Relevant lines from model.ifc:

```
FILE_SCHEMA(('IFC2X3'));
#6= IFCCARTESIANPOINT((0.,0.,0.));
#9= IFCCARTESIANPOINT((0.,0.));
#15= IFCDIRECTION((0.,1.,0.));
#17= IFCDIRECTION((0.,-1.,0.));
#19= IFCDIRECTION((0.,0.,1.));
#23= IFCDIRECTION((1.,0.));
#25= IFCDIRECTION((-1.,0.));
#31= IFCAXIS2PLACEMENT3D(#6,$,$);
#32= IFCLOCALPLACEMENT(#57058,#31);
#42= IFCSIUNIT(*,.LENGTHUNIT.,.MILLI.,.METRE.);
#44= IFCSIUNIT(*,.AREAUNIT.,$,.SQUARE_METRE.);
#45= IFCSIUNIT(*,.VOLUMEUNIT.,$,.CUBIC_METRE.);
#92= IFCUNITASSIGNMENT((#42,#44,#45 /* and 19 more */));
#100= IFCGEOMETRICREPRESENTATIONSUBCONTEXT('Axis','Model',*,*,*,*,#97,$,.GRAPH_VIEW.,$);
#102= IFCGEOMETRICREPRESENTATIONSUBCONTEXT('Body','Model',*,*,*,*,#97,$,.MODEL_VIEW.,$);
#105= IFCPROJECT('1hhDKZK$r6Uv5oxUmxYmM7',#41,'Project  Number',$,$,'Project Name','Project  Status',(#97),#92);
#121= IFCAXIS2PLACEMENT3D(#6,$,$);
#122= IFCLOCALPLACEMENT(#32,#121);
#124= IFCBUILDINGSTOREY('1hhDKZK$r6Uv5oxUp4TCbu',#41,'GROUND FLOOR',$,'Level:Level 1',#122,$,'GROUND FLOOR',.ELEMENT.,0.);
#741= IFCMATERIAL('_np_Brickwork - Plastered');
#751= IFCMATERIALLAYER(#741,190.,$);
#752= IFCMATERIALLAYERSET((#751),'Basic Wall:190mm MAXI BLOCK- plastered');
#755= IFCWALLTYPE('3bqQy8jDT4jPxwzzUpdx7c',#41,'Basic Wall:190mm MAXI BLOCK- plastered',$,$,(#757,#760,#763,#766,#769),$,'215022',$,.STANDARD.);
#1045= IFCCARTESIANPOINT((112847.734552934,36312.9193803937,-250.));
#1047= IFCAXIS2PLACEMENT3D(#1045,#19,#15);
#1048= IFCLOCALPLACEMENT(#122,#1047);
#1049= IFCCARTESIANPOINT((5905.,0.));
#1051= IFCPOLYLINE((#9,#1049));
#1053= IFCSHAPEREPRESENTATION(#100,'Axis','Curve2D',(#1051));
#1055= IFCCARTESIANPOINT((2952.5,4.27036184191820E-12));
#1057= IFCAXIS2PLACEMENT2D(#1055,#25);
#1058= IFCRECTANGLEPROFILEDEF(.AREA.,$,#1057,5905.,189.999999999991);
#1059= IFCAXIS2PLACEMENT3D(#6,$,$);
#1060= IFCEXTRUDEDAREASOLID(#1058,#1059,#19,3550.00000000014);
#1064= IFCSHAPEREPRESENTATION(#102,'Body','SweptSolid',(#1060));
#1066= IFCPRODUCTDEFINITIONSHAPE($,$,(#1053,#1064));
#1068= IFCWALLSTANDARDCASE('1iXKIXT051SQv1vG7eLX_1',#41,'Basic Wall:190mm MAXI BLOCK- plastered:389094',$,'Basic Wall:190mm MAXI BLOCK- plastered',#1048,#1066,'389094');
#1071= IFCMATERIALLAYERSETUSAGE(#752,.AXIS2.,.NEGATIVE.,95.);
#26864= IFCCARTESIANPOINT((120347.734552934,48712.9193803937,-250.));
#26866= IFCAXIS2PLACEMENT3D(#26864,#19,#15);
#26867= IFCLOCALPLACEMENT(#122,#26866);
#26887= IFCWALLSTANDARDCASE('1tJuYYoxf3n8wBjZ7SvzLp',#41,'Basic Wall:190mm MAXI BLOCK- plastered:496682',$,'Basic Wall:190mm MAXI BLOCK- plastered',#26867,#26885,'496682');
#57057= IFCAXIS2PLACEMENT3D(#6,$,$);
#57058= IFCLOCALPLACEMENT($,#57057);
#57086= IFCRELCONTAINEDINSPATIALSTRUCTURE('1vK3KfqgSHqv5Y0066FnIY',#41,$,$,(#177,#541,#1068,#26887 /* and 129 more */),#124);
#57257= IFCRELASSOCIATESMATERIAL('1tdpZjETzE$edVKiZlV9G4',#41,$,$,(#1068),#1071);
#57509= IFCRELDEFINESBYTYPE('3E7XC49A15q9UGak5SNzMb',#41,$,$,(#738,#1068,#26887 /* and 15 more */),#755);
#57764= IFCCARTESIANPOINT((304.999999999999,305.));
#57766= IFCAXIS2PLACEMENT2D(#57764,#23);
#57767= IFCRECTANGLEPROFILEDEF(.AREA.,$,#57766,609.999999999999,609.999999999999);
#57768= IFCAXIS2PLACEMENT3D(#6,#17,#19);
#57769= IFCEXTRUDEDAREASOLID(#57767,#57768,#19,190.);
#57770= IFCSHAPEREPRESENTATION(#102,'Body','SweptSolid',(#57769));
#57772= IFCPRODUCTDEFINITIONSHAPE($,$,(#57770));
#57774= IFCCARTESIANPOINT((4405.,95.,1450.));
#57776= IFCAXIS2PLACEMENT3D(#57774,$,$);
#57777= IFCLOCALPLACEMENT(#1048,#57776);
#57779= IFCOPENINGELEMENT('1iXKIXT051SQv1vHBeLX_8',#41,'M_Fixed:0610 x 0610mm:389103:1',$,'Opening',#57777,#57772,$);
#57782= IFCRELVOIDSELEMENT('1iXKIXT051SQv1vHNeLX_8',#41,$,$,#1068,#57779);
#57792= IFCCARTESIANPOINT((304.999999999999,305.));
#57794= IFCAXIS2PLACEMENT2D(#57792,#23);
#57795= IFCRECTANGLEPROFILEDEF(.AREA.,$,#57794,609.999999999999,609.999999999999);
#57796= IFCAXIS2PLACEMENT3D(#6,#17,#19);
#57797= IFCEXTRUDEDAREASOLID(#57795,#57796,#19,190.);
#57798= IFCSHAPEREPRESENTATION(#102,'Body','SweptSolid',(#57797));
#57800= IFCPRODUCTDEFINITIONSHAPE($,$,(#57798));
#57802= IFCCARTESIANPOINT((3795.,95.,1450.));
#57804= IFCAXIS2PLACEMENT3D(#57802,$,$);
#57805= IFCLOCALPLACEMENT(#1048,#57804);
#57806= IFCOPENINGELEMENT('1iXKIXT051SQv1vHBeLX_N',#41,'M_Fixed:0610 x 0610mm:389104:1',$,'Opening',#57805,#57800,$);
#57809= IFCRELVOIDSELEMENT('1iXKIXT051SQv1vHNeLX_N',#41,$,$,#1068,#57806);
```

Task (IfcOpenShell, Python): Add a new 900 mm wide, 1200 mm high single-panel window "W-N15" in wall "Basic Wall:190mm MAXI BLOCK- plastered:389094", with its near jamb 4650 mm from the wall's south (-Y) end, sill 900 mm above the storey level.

```python
import numpy as np
import ifcopenshell
import ifcopenshell.api.feature
import ifcopenshell.api.geometry
import ifcopenshell.api.root
import ifcopenshell.api.spatial
import ifcopenshell.api.type
import ifcopenshell.geom
import ifcopenshell.util.element
import ifcopenshell.util.placement
import ifcopenshell.util.representation
import ifcopenshell.util.shape
import ifcopenshell.util.unit

model = ifcopenshell.open("model.ifc")
unit_scale = ifcopenshell.util.unit.calculate_unit_scale(model)
settings = ifcopenshell.geom.settings()


def volume(element):
    """Net volume in cubic metres, openings subtracted."""
    shape = ifcopenshell.geom.create_shape(settings, element)
    return ifcopenshell.util.shape.get_volume(shape.geometry)


wall = model.by_guid("1iXKIXT051SQv1vG7eLX_1")
storey = ifcopenshell.util.element.get_container(wall, ifc_class="IfcBuildingStorey")
context = ifcopenshell.util.representation.get_context(model, "Model", "Body", "MODEL_VIEW")
before = volume(wall)

width, height, from_end, sill = 0.9, 1.2, 4.65, 0.9  # metres

# The wall runs along its own X axis, and the end named is its -X end.
wall_shape = ifcopenshell.geom.create_shape(settings, wall)
x, y, z = ifcopenshell.util.shape.get_vertices(wall_shape.geometry).T
start = x.min() + from_end
face, thickness = float(y.min()), float(y.max() - y.min())
wall_matrix = ifcopenshell.util.placement.get_local_placement(wall.ObjectPlacement)
level = ifcopenshell.util.placement.get_local_placement(storey.ObjectPlacement)[2, 3]


def in_wall(x, y):
    """Placement at x, y metres in the wall's axes, at sill height."""
    matrix = wall_matrix.copy()
    matrix[:, 3] = wall_matrix @ np.array([x / unit_scale, y / unit_scale, 0.0, 1.0])
    matrix[2, 3] = level + sill / unit_scale
    return matrix


# Opening: a box that overshoots both wall faces by 50 mm.
opening = ifcopenshell.api.root.create_entity(model, ifc_class="IfcOpeningElement")
box = ifcopenshell.api.geometry.add_wall_representation(
    model, context=context, length=width, height=height, thickness=thickness + 0.1
)
ifcopenshell.api.geometry.assign_representation(model, product=opening, representation=box)
ifcopenshell.api.geometry.edit_object_placement(model, product=opening, matrix=in_wall(start, face - 0.05), is_si=False)
ifcopenshell.api.feature.add_feature(model, feature=opening, element=wall)

window = ifcopenshell.api.root.create_entity(model, ifc_class="IfcWindow", name="W-N15")
window.OverallWidth, window.OverallHeight = width / unit_scale, height / unit_scale
body = ifcopenshell.api.geometry.add_window_representation(
    model,
    context=context,
    overall_width=window.OverallWidth,
    overall_height=window.OverallHeight,
    partition_type="SINGLE_PANEL",
)
ifcopenshell.api.geometry.assign_representation(model, product=window, representation=body)
ifcopenshell.api.spatial.assign_container(model, products=[window], relating_structure=storey)
fills = ifcopenshell.api.feature.add_filling(model, opening=opening, element=window)
fills.OwnerHistory = window.OwnerHistory  # required in IFC2X3

# IFC2X3 keeps the operation on the window style.
style = ifcopenshell.api.root.create_entity(model, ifc_class="IfcWindowStyle", name="W-N15")
style.OperationType, style.ConstructionType = "SINGLE_PANEL", "NOTDEFINED"
style.ParameterTakesPrecedence = style.Sizeable = False
ifcopenshell.api.type.assign_type(model, related_objects=[window], relating_type=style)

# Centre the window in the wall's thickness.
ifcopenshell.api.geometry.edit_object_placement(model, product=window, matrix=in_wall(start, face), is_si=False)
window_shape = ifcopenshell.geom.create_shape(settings, window)
depth = ifcopenshell.util.shape.get_vertices(window_shape.geometry)[:, 1]
offset = face + thickness / 2 - (depth.min() + depth.max()) / 2
ifcopenshell.api.geometry.edit_object_placement(model, product=window, matrix=in_wall(start, offset), is_si=False)

after = volume(wall)

print(f"wall volume {before:.3f} -> {after:.3f} m3")

model.write("model_edited.ifc")
```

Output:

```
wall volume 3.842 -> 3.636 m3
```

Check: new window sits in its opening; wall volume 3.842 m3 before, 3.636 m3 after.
